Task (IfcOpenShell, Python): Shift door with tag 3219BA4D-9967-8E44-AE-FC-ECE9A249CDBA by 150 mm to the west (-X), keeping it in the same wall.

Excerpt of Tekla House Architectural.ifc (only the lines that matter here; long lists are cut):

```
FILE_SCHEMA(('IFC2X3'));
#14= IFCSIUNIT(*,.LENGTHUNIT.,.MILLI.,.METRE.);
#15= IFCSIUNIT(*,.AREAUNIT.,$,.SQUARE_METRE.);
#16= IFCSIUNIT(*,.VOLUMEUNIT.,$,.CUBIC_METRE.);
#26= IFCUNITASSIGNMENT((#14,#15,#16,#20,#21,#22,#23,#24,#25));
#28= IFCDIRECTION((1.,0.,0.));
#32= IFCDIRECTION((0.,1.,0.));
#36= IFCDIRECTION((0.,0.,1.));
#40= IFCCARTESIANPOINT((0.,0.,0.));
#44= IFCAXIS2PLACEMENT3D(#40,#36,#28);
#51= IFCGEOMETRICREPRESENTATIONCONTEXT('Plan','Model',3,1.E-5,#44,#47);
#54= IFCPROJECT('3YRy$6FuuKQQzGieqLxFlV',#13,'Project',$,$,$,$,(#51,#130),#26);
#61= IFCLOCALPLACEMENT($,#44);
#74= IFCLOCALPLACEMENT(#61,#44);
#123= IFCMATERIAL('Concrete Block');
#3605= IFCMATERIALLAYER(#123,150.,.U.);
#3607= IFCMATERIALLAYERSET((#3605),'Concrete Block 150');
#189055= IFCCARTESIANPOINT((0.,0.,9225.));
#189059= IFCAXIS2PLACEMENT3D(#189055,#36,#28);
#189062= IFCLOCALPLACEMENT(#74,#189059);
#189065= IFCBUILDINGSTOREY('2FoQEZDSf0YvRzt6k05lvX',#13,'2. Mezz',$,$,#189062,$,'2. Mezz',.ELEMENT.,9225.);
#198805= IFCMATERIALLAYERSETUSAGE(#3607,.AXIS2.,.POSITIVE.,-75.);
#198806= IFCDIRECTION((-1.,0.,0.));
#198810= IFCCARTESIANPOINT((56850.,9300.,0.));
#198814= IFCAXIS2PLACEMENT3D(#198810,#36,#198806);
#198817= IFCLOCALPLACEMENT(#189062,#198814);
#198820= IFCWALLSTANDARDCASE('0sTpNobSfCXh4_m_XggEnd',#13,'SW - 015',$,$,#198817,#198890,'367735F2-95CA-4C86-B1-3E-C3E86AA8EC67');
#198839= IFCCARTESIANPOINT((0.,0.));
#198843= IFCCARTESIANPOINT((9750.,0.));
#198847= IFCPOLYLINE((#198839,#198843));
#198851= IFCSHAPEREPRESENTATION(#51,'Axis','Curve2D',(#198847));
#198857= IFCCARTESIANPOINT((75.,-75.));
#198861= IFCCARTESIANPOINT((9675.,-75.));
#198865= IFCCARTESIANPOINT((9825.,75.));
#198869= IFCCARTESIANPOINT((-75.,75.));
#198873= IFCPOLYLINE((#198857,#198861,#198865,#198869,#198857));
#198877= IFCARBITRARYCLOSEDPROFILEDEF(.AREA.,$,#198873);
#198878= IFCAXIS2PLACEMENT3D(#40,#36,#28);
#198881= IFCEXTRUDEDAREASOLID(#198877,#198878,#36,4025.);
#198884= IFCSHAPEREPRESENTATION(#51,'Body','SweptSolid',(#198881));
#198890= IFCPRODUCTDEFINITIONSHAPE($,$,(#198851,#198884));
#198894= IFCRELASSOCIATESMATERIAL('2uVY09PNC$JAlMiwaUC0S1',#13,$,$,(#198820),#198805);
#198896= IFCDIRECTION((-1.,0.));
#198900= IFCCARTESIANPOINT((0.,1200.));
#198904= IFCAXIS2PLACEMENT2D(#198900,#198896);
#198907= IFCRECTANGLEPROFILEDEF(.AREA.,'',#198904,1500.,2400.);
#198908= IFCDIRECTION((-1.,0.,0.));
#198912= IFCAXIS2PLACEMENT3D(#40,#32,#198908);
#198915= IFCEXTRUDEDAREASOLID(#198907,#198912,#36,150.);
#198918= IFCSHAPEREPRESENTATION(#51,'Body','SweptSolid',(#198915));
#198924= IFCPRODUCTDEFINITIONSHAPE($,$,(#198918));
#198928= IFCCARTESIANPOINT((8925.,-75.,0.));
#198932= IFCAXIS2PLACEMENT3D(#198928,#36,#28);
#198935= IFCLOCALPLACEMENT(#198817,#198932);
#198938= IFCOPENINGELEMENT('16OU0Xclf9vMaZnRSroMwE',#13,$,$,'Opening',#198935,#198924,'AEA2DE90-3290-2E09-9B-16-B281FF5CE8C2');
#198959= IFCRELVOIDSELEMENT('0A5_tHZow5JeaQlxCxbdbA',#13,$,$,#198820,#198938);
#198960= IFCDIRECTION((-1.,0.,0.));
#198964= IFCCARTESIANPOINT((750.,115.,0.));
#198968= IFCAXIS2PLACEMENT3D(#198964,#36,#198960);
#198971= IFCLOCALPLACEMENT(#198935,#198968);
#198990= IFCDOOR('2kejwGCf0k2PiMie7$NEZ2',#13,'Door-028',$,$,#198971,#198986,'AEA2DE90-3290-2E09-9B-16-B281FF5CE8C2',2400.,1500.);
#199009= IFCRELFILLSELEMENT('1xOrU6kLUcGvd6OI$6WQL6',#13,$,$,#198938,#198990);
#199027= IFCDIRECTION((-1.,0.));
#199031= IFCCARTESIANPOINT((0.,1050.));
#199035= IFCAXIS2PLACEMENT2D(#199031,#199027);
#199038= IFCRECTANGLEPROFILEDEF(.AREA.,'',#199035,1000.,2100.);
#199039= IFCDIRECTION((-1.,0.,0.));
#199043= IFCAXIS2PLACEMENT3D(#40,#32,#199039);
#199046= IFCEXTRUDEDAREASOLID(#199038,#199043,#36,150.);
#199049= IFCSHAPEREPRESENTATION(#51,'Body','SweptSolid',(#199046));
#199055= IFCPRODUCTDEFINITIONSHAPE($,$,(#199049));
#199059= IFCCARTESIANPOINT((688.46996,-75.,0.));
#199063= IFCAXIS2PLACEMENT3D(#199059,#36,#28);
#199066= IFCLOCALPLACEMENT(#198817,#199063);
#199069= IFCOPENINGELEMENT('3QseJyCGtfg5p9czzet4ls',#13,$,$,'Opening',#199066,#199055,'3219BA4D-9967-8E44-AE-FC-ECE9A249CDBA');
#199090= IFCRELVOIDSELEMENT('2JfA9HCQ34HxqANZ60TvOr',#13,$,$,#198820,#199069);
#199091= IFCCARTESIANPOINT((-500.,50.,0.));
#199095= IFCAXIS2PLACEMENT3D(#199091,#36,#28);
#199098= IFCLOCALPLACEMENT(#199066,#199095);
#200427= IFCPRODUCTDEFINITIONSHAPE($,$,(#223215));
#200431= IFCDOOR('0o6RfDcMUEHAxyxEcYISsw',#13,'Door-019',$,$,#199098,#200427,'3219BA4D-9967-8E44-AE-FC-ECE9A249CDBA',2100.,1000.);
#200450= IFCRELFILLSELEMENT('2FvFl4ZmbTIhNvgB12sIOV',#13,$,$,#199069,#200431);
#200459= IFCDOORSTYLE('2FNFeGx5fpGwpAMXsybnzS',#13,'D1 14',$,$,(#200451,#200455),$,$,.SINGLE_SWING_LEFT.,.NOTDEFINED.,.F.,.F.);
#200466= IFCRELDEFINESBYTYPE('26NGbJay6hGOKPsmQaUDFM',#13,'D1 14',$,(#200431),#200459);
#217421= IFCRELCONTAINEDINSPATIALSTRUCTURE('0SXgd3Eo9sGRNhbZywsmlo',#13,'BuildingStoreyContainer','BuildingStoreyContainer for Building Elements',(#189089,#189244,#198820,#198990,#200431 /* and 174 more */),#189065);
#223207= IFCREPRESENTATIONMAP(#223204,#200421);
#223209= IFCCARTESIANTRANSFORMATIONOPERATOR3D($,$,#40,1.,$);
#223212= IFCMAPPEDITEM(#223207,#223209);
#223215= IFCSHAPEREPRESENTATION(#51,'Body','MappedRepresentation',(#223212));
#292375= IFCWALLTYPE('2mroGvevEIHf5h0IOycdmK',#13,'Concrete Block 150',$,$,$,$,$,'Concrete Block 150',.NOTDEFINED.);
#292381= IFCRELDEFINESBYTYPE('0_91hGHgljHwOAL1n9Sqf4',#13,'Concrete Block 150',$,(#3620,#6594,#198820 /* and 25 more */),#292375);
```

```python
import ifcopenshell
import ifcopenshell.api.geometry
import ifcopenshell.util.placement
import ifcopenshell.util.unit

model = ifcopenshell.open("Tekla House Architectural.ifc")
unit_scale = ifcopenshell.util.unit.calculate_unit_scale(model)

door = model.by_guid("0o6RfDcMUEHAxyxEcYISsw")
opening = door.FillsVoids[0].RelatingOpeningElement
wall = opening.VoidsElements[0].RelatingBuildingElement

wall_matrix = ifcopenshell.util.placement.get_local_placement(wall.ObjectPlacement)
shift = wall_matrix[:3, 0] * 0.15 / unit_scale
before = ifcopenshell.util.placement.get_local_placement(door.ObjectPlacement)[:3, 3].copy()

# The door is placed relative to its opening, so it follows when the opening moves.
matrix = ifcopenshell.util.placement.get_local_placement(opening.ObjectPlacement)
matrix[:3, 3] += shift
ifcopenshell.api.geometry.edit_object_placement(
    model, product=opening, matrix=matrix, is_si=False, should_transform_children=True
)

after = ifcopenshell.util.placement.get_local_placement(door.ObjectPlacement)[:3, 3]
print("door moved by", (after - before).round(3) + 0.0)

model.write("Tekla House Architectural_edited.ifc")
```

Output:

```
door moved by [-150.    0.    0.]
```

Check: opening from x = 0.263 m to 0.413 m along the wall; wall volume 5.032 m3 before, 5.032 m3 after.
